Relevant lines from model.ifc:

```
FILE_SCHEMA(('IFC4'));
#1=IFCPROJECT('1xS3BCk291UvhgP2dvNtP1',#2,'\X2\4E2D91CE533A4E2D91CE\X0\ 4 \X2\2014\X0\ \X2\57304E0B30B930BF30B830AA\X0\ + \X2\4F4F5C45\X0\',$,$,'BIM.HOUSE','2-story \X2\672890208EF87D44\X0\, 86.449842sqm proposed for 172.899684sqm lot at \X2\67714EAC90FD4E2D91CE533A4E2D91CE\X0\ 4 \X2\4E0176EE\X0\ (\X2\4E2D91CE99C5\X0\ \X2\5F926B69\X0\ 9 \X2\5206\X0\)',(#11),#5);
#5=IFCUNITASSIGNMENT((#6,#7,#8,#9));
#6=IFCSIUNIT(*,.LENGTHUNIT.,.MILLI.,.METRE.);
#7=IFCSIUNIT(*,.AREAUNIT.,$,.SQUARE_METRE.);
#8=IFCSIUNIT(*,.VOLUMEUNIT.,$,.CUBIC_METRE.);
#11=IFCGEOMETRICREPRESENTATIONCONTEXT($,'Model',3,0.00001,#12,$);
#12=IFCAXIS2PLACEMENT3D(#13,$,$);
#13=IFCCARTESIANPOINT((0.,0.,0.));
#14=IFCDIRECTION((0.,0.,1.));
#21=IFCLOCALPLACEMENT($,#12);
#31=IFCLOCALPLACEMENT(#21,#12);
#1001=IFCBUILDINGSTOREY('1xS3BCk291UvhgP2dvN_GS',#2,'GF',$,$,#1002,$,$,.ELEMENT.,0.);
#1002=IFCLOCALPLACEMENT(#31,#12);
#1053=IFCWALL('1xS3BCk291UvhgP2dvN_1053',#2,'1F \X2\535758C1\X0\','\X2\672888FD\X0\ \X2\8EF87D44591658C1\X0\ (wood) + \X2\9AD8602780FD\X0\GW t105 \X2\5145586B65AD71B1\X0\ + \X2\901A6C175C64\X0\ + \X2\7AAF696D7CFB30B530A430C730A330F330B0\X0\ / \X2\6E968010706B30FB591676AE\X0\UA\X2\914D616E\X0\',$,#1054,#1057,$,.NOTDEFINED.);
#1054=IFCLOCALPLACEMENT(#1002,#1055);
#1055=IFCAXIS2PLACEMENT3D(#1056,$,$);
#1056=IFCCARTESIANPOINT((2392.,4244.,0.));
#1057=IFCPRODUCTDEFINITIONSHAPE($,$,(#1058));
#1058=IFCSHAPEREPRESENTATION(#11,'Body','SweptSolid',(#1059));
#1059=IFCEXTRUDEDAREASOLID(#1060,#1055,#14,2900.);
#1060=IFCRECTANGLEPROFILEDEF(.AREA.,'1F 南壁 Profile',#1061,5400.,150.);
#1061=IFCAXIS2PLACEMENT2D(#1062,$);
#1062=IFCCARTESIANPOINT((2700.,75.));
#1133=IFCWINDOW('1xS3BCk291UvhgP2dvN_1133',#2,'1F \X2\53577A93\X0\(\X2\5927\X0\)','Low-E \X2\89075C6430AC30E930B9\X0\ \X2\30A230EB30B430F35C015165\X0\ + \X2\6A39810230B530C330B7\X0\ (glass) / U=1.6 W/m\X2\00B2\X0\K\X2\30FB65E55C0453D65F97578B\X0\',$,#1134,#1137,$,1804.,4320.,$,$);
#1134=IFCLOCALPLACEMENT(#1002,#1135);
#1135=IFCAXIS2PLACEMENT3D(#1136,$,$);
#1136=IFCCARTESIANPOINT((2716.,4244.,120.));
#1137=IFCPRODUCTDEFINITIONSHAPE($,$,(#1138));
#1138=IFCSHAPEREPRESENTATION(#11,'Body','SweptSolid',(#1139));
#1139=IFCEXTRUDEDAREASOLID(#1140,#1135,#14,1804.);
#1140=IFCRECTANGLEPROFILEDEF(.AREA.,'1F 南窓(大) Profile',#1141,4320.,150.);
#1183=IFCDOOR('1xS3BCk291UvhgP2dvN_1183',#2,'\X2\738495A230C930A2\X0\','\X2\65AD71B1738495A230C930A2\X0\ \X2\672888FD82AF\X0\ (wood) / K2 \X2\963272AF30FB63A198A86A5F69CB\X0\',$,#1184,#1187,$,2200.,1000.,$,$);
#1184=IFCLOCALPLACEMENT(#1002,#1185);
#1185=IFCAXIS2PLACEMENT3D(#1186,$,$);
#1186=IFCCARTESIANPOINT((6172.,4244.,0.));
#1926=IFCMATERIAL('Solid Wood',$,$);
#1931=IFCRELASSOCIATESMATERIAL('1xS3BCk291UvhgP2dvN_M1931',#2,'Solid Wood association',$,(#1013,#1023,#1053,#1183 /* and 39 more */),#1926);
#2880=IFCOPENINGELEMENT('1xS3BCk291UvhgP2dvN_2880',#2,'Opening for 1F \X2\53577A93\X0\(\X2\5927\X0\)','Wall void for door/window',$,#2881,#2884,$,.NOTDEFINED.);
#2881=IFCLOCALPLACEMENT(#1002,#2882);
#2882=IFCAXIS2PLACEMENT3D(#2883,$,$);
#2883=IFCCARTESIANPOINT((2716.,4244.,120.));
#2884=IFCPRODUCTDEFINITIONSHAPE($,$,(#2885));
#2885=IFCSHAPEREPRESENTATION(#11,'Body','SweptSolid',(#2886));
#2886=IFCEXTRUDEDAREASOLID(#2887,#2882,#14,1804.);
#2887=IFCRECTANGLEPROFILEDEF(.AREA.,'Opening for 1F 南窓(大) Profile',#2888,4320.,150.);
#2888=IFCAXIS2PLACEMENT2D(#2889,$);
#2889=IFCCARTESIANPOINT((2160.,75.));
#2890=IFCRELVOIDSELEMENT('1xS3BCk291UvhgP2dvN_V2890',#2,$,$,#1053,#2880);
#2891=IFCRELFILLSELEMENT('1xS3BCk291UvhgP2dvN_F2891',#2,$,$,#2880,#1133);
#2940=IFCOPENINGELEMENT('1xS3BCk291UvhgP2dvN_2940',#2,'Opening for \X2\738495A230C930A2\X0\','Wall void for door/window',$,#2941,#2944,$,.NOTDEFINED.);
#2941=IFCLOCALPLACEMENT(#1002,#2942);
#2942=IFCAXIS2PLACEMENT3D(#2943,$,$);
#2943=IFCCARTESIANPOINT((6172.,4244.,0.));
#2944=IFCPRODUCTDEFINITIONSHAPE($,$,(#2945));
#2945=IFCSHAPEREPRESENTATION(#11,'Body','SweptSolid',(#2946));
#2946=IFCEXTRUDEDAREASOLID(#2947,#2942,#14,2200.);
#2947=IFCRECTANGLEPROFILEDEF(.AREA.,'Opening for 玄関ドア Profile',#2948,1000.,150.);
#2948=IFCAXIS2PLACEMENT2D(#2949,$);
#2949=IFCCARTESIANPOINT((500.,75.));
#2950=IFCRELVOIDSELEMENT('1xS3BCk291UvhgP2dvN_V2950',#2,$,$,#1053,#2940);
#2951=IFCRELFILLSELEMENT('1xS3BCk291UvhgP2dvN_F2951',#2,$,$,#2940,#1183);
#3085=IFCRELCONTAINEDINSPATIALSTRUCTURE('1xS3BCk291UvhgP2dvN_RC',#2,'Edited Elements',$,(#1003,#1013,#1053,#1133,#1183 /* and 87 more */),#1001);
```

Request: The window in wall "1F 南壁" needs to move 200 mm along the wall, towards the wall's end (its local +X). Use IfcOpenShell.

```python
import ifcopenshell
import ifcopenshell.api.geometry
import ifcopenshell.util.placement

model = ifcopenshell.open("model.ifc")

window = model.by_guid("1xS3BCk291UvhgP2dvN_1133")
opening = window.FillsVoids[0].RelatingOpeningElement
wall = opening.VoidsElements[0].RelatingBuildingElement

wall_matrix = ifcopenshell.util.placement.get_local_placement(wall.ObjectPlacement)
shift = wall_matrix[:3, 0] * 200.0
before = ifcopenshell.util.placement.get_local_placement(window.ObjectPlacement)[:3, 3].copy()

# The window is not placed relative to its opening, so move both.
for product in (opening, window):
    matrix = ifcopenshell.util.placement.get_local_placement(product.ObjectPlacement)
    matrix[:3, 3] += shift
    ifcopenshell.api.geometry.edit_object_placement(model, product=product, matrix=matrix, is_si=False)

after = ifcopenshell.util.placement.get_local_placement(window.ObjectPlacement)[:3, 3]
print("window moved by", (after - before).round(3) + 0.0)

model.write("model_edited.ifc")
```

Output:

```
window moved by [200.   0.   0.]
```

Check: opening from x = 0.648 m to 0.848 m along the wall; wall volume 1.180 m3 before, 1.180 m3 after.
